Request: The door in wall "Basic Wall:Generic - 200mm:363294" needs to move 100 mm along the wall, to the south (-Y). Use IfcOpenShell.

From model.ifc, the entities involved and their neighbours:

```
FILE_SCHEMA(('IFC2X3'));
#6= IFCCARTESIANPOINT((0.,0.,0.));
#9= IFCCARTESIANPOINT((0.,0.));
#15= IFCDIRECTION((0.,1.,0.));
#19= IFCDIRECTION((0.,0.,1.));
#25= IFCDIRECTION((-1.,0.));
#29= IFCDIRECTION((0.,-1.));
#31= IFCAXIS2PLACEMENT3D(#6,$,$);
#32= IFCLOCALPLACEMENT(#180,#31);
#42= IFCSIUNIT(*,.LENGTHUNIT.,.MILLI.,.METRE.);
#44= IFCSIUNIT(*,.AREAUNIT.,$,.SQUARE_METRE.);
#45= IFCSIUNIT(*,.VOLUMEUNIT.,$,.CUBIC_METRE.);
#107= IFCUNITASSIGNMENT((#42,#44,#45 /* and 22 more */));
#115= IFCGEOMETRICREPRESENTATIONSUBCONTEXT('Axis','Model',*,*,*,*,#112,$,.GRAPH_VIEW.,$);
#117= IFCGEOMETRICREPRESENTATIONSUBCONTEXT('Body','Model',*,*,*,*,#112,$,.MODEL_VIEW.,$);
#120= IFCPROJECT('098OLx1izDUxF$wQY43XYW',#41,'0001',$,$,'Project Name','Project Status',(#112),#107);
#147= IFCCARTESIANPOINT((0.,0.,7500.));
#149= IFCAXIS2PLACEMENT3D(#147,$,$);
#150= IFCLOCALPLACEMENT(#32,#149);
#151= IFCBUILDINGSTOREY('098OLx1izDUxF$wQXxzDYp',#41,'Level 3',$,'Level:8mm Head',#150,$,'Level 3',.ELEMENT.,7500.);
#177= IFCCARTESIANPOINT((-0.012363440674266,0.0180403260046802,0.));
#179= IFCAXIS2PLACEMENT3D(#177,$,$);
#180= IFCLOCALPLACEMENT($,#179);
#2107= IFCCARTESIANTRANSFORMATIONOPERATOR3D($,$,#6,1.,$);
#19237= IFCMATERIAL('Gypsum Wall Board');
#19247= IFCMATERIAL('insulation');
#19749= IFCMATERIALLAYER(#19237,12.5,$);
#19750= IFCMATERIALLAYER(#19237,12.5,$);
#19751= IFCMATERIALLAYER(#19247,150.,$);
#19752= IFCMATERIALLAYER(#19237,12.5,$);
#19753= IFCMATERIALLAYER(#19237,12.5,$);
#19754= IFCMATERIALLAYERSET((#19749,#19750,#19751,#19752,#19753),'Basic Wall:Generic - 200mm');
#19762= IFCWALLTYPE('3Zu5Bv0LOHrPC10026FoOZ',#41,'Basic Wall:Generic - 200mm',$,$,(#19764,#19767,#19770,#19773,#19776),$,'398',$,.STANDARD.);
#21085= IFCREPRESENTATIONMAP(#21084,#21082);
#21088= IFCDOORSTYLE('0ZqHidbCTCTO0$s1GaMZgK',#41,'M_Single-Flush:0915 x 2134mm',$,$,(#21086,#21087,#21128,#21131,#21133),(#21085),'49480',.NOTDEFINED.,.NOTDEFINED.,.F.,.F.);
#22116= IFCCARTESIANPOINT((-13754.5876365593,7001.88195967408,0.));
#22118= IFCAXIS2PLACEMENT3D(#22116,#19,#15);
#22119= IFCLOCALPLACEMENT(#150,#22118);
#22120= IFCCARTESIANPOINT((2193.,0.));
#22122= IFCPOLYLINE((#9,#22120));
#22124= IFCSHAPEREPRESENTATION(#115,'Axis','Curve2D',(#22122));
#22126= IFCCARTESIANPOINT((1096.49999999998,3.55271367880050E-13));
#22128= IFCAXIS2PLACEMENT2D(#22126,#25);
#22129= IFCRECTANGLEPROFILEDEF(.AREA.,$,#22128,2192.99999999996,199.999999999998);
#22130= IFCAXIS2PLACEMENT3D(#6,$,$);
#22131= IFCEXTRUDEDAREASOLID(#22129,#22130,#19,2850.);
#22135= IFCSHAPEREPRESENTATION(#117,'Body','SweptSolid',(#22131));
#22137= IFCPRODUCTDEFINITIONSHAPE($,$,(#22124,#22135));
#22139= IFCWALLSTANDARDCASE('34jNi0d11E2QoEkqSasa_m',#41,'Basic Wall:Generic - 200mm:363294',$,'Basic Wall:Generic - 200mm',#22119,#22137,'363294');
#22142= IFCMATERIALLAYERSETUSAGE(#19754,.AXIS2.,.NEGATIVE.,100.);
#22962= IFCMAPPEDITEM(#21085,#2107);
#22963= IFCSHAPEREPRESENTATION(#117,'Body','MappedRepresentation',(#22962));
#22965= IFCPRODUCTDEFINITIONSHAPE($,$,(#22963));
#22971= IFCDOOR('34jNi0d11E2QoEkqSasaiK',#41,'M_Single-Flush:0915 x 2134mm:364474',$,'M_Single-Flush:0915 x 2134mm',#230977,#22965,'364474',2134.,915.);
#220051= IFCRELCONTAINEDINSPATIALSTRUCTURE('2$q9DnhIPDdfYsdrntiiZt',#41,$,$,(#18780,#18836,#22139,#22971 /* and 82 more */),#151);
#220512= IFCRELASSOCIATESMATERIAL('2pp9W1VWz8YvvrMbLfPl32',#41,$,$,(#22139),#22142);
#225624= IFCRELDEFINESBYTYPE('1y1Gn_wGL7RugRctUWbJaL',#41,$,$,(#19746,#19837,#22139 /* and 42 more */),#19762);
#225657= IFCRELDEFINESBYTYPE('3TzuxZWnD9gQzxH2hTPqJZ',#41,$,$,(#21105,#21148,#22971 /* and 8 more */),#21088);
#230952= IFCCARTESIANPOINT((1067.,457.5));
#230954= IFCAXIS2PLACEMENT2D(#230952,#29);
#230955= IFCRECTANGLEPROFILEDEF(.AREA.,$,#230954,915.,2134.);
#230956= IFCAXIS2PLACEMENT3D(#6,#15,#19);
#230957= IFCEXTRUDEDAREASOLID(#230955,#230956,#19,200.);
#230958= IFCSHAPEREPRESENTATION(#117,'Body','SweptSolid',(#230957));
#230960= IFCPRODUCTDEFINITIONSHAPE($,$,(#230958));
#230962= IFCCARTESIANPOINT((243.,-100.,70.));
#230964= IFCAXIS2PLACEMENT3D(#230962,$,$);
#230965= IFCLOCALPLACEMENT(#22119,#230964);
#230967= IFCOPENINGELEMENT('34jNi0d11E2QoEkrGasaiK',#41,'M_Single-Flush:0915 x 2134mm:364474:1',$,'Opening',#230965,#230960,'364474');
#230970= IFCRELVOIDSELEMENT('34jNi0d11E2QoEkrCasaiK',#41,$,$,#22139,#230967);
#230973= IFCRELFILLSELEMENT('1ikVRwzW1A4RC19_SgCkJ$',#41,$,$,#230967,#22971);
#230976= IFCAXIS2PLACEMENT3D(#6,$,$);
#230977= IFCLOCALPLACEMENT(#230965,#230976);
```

```python
import ifcopenshell
import ifcopenshell.api.geometry
import ifcopenshell.util.placement
import ifcopenshell.util.unit

model = ifcopenshell.open("model.ifc")
unit_scale = ifcopenshell.util.unit.calculate_unit_scale(model)

door = model.by_guid("34jNi0d11E2QoEkqSasaiK")
opening = door.FillsVoids[0].RelatingOpeningElement
wall = opening.VoidsElements[0].RelatingBuildingElement

wall_matrix = ifcopenshell.util.placement.get_local_placement(wall.ObjectPlacement)
shift = wall_matrix[:3, 0] * -0.1 / unit_scale
before = ifcopenshell.util.placement.get_local_placement(door.ObjectPlacement)[:3, 3].copy()

# The door is placed relative to its opening, so it follows when the opening moves.
matrix = ifcopenshell.util.placement.get_local_placement(opening.ObjectPlacement)
matrix[:3, 3] += shift
ifcopenshell.api.geometry.edit_object_placement(
    model, product=opening, matrix=matrix, is_si=False, should_transform_children=True
)

after = ifcopenshell.util.placement.get_local_placement(door.ObjectPlacement)[:3, 3]
print("door moved by", (after - before).round(3) + 0.0)

model.write("model_edited.ifc")
```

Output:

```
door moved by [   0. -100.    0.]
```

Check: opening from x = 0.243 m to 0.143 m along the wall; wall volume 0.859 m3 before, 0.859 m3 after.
